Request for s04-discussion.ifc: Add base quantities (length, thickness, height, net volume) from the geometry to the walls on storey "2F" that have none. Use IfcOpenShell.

First a look at what the model holds.

```python
import ifcopenshell
import ifcopenshell.util.element
import ifcopenshell.util.unit

model = ifcopenshell.open("s04-discussion.ifc")
print(model.schema)
for unit_type in ("LENGTHUNIT", "AREAUNIT", "VOLUMEUNIT"):
    print(unit_type, ifcopenshell.util.unit.calculate_unit_scale(model, unit_type))
storey = next(s for s in model.by_type("IfcBuildingStorey") if s.Name == "2F")
walls = [e for e in ifcopenshell.util.element.get_decomposition(storey) if e.is_a("IfcWall")]
for e in sorted(walls, key=lambda e: e.id()):
    print(e.id(), e.is_a(), e.Name, list(ifcopenshell.util.element.get_psets(e, qtos_only=True)), sep=" | ")
```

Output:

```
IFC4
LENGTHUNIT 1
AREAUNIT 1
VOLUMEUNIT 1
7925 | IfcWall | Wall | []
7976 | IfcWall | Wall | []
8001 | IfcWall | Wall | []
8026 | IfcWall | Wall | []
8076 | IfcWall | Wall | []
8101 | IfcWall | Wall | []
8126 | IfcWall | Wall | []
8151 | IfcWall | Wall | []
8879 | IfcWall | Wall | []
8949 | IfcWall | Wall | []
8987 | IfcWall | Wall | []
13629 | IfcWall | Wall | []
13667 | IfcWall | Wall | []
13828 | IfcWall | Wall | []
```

```python
import ifcopenshell
import ifcopenshell.api.pset
import ifcopenshell.geom
import ifcopenshell.util.element
import ifcopenshell.util.shape
import ifcopenshell.util.unit

model = ifcopenshell.open("s04-discussion.ifc")
unit_scale = ifcopenshell.util.unit.calculate_unit_scale(model)
volume_scale = ifcopenshell.util.unit.calculate_unit_scale(model, "VOLUMEUNIT")
settings = ifcopenshell.geom.settings()

storey = next(s for s in model.by_type("IfcBuildingStorey") if s.Name == "2F")
walls = [e for e in ifcopenshell.util.element.get_decomposition(storey) if e.is_a("IfcWall")]

for e in sorted(walls, key=lambda e: e.id()):
    if ifcopenshell.util.element.get_psets(e, qtos_only=True, should_inherit=False):
        continue
    # Geometry comes back in metres, in the element's own axes.
    shape = ifcopenshell.geom.create_shape(settings, e)
    values = {
        "Length": ifcopenshell.util.shape.get_x(shape.geometry) / unit_scale,
        "Width": ifcopenshell.util.shape.get_y(shape.geometry) / unit_scale,
        "Height": ifcopenshell.util.shape.get_z(shape.geometry) / unit_scale,
        "NetVolume": ifcopenshell.util.shape.get_volume(shape.geometry) / volume_scale,
    }
    qto = ifcopenshell.api.pset.add_qto(model, product=e, name="Qto_WallBaseQuantities")
    ifcopenshell.api.pset.edit_qto(model, qto=qto, properties=values)
    print(e.id(), {k: round(v, 3) for k, v in values.items()})

model.write("s04-discussion_updated.ifc")
```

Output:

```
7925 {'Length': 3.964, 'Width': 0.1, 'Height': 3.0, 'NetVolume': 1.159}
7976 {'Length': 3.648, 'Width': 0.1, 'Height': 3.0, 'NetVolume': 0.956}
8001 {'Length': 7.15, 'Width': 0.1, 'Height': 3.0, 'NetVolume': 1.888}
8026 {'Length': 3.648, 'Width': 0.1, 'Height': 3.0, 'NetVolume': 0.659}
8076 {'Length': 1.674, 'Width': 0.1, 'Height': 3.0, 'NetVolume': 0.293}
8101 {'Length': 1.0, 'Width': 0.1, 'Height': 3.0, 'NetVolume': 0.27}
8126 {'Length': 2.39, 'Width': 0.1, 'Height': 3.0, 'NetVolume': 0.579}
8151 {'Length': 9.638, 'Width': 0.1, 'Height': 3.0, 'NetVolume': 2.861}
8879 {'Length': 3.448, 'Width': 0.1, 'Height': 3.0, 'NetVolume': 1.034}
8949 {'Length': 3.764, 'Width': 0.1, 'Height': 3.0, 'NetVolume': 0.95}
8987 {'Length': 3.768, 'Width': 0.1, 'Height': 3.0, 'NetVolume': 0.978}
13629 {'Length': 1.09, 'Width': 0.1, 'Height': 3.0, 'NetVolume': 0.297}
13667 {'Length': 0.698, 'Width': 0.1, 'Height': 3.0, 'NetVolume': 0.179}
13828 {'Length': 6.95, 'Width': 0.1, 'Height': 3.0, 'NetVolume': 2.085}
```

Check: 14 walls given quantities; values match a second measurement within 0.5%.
